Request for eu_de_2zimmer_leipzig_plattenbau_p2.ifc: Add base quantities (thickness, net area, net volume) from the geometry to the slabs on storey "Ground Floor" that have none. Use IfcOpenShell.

First a look at what the model holds.

```python
import ifcopenshell
import ifcopenshell.util.element
import ifcopenshell.util.unit

model = ifcopenshell.open("eu_de_2zimmer_leipzig_plattenbau_p2.ifc")
print(model.schema)
for unit_type in ("LENGTHUNIT", "AREAUNIT", "VOLUMEUNIT"):
    print(unit_type, ifcopenshell.util.unit.calculate_unit_scale(model, unit_type))
storey = next(s for s in model.by_type("IfcBuildingStorey") if s.Name == "Ground Floor")
slabs = [e for e in ifcopenshell.util.element.get_decomposition(storey) if e.is_a("IfcSlab")]
for e in sorted(slabs, key=lambda e: e.id()):
    print(e.id(), e.is_a(), e.Name, list(ifcopenshell.util.element.get_psets(e, qtos_only=True)), sep=" | ")
```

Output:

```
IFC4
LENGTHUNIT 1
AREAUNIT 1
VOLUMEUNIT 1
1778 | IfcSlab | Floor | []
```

```python
import ifcopenshell
import ifcopenshell.api.pset
import ifcopenshell.geom
import ifcopenshell.util.element
import ifcopenshell.util.shape
import ifcopenshell.util.unit

model = ifcopenshell.open("eu_de_2zimmer_leipzig_plattenbau_p2.ifc")
unit_scale = ifcopenshell.util.unit.calculate_unit_scale(model)
area_scale = ifcopenshell.util.unit.calculate_unit_scale(model, "AREAUNIT")
volume_scale = ifcopenshell.util.unit.calculate_unit_scale(model, "VOLUMEUNIT")
settings = ifcopenshell.geom.settings()

storey = next(s for s in model.by_type("IfcBuildingStorey") if s.Name == "Ground Floor")
slabs = [e for e in ifcopenshell.util.element.get_decomposition(storey) if e.is_a("IfcSlab")]

for e in sorted(slabs, key=lambda e: e.id()):
    if ifcopenshell.util.element.get_psets(e, qtos_only=True, should_inherit=False):
        continue
    # Geometry comes back in metres, in the element's own axes.
    shape = ifcopenshell.geom.create_shape(settings, e)
    values = {
        "Width": ifcopenshell.util.shape.get_z(shape.geometry) / unit_scale,
        "NetArea": ifcopenshell.util.shape.get_footprint_area(shape.geometry) / area_scale,
        "NetVolume": ifcopenshell.util.shape.get_volume(shape.geometry) / volume_scale,
    }
    qto = ifcopenshell.api.pset.add_qto(model, product=e, name="Qto_SlabBaseQuantities")
    ifcopenshell.api.pset.edit_qto(model, qto=qto, properties=values)
    print(e.id(), {k: round(v, 3) for k, v in values.items()})

model.write("eu_de_2zimmer_leipzig_plattenbau_p2_v2.ifc")
```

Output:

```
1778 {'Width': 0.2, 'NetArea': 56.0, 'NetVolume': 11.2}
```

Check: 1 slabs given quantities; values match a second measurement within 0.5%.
